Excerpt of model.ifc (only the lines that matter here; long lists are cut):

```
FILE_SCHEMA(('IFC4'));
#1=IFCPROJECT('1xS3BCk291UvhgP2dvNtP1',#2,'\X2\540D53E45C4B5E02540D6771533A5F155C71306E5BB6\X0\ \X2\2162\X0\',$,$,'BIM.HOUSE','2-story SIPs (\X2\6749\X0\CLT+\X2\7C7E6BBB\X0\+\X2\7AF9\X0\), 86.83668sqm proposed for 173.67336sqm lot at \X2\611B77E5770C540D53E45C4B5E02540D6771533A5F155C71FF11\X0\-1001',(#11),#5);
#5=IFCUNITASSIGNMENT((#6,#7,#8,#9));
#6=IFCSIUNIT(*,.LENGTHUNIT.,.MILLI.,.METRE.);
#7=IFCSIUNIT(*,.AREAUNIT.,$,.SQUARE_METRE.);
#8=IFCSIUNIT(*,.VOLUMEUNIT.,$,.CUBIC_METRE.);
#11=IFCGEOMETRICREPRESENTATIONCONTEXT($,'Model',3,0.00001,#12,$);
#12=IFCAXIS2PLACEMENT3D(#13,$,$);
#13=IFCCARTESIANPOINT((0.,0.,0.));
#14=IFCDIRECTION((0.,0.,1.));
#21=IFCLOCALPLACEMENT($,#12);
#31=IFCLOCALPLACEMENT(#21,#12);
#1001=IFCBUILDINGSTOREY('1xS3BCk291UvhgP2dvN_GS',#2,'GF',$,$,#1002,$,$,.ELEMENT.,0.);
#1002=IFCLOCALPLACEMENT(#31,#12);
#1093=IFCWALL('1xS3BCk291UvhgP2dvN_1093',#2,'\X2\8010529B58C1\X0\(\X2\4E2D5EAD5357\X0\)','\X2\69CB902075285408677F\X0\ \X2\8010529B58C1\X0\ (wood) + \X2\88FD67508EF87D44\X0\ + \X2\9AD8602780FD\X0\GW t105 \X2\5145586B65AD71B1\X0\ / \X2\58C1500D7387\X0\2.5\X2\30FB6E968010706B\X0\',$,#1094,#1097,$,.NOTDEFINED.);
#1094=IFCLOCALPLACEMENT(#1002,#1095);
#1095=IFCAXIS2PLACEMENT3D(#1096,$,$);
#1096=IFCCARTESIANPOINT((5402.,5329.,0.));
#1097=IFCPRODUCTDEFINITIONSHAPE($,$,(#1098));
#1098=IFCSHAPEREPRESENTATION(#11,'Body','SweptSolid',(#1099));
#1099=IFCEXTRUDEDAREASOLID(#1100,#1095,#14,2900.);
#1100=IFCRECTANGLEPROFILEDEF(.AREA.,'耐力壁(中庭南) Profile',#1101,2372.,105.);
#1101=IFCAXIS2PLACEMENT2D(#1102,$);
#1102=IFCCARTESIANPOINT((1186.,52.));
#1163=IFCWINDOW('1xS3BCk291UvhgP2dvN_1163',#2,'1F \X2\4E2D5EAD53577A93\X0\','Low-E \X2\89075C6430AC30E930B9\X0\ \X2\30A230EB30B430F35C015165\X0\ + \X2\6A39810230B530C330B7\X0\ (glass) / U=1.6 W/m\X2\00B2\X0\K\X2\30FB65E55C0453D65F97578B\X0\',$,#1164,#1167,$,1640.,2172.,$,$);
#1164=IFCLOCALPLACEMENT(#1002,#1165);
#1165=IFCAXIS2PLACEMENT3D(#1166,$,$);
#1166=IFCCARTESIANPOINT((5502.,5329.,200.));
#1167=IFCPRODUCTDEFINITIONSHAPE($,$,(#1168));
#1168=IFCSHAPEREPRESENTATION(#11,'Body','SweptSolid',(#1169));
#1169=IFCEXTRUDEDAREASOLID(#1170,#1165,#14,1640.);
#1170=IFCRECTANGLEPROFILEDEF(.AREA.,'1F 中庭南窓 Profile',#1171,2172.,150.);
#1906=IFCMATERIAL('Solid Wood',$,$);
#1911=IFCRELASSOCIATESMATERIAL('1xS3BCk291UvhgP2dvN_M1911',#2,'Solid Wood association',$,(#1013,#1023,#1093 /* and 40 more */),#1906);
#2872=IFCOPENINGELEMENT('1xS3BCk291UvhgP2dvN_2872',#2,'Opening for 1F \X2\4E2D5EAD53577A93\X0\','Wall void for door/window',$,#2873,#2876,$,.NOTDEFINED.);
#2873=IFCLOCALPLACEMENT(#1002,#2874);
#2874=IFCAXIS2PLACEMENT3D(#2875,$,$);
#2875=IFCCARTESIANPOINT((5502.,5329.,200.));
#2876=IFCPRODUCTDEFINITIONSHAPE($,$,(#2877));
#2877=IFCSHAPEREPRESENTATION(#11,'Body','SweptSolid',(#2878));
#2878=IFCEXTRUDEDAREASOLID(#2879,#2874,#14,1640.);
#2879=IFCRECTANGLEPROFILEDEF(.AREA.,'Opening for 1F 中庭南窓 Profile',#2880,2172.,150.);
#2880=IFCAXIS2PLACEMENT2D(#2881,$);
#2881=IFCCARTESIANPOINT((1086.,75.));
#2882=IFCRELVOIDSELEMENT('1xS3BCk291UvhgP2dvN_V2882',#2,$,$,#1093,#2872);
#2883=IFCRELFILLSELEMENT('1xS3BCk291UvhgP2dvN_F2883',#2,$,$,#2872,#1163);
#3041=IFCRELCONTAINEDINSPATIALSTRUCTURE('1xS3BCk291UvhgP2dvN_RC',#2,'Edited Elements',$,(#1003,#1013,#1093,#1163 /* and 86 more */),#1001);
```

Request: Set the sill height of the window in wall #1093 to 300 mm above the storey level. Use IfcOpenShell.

```python
import numpy as np
import ifcopenshell
import ifcopenshell.api.geometry
import ifcopenshell.geom
import ifcopenshell.util.element
import ifcopenshell.util.placement
import ifcopenshell.util.shape
import ifcopenshell.util.unit

model = ifcopenshell.open("model.ifc")
unit_scale = ifcopenshell.util.unit.calculate_unit_scale(model)

window = model.by_guid("1xS3BCk291UvhgP2dvN_1163")
opening = window.FillsVoids[0].RelatingOpeningElement
storey = ifcopenshell.util.element.get_container(window, ifc_class="IfcBuildingStorey")
level = ifcopenshell.util.placement.get_local_placement(storey.ObjectPlacement)[2, 3]

# The opening's origin need not be at the sill, so measure its lowest point.
shape = ifcopenshell.geom.create_shape(ifcopenshell.geom.settings(), opening)
bottom = ifcopenshell.util.shape.get_shape_bottom_elevation(shape, shape.geometry) / unit_scale
dz = level + 0.3 / unit_scale - bottom

shift = np.array([0.0, 0.0, dz])
# The window is not placed relative to its opening, so move both.
for product in (opening, window):
    matrix = ifcopenshell.util.placement.get_local_placement(product.ObjectPlacement)
    matrix[:3, 3] += shift
    ifcopenshell.api.geometry.edit_object_placement(model, product=product, matrix=matrix, is_si=False)

print(f"moved by {dz * unit_scale:+.3f} m")

model.write("model_updated.ifc")
```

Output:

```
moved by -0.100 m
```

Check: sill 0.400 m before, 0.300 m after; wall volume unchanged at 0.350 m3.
